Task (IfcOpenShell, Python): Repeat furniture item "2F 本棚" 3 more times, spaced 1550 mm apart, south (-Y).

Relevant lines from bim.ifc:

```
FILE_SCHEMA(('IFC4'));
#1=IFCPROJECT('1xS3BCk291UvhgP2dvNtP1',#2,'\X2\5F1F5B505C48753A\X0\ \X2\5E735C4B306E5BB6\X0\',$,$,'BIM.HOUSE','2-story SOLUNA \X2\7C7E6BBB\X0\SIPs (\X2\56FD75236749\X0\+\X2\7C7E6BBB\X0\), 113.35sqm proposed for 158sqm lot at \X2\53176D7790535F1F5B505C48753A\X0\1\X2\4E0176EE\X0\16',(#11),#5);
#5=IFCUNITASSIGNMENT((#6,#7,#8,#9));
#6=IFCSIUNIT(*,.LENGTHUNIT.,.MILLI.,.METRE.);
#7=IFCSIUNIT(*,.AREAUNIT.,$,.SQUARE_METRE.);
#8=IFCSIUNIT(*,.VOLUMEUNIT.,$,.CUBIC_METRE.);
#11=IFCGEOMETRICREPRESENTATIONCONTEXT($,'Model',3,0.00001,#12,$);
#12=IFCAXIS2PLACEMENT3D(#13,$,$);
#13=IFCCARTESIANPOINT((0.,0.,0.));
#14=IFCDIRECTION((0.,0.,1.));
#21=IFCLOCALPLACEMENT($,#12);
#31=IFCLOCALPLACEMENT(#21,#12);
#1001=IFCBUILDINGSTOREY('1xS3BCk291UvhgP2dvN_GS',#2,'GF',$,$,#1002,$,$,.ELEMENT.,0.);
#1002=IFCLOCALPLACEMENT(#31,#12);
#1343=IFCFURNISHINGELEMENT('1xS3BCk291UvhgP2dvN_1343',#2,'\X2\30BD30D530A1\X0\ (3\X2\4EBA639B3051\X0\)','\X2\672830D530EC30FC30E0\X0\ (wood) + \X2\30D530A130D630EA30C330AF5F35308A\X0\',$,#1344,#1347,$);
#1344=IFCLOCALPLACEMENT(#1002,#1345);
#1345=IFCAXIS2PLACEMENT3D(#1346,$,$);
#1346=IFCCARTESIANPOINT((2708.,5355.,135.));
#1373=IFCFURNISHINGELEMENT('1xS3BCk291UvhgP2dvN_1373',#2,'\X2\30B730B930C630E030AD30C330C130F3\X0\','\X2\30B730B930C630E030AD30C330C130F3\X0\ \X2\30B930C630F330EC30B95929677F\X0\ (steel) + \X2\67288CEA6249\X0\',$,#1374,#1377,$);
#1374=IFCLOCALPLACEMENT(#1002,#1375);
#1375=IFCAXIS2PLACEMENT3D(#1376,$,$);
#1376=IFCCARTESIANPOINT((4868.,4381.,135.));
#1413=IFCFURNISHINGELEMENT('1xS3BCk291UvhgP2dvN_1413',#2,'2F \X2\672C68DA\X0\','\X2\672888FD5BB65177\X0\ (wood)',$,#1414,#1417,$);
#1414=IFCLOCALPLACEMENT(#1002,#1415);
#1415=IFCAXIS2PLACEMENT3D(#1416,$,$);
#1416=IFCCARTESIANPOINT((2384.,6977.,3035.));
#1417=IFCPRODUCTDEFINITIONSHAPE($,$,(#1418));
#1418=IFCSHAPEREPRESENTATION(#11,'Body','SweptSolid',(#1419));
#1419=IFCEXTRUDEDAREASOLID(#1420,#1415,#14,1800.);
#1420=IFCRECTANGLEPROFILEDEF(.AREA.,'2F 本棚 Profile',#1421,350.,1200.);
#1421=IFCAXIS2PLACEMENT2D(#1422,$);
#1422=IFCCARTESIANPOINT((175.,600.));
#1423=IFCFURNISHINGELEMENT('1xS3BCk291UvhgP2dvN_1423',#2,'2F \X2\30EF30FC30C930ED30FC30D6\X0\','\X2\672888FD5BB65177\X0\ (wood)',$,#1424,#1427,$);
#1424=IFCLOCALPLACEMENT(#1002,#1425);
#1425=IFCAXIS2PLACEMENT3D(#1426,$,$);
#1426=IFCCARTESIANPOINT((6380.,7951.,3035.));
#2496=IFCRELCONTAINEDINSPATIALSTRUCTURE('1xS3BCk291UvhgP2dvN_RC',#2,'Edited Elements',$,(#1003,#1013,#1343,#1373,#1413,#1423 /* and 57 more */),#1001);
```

```python
import numpy as np
import ifcopenshell
import ifcopenshell.api.geometry
import ifcopenshell.api.root
import ifcopenshell.util.element
import ifcopenshell.util.placement

model = ifcopenshell.open("bim.ifc")


def reuse_history(source, copy):
    """copy_class also copies each property set's owner history, people and application; keep the originals."""
    for rel in copy.IsDefinedBy:
        if rel.is_a("IfcRelDefinesByProperties") and (history := rel.RelatingPropertyDefinition.OwnerHistory):
            rel.RelatingPropertyDefinition.OwnerHistory = source.OwnerHistory
            ifcopenshell.util.element.remove_deep2(model, history)


source = model.by_guid("1xS3BCk291UvhgP2dvN_1413")
base = ifcopenshell.util.placement.get_local_placement(source.ObjectPlacement)
step = np.array([0.0, -1.0, 0.0]) * 1550.0

for i in range(1, 4):
    copy = ifcopenshell.api.root.copy_class(model, product=source)
    copy.Representation = ifcopenshell.util.element.copy_deep(
        model, source.Representation, exclude=["IfcGeometricRepresentationContext", "IfcRepresentationMap"]
    )
    reuse_history(source, copy)
    matrix = base.copy()
    matrix[:3, 3] += i * step
    print("added at", matrix[:3, 3].round(3) + 0.0)
    ifcopenshell.api.geometry.edit_object_placement(model, product=copy, matrix=matrix, is_si=False)

model.write("bim-out.ifc")
```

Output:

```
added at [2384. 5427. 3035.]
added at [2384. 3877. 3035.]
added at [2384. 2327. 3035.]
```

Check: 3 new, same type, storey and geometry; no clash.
